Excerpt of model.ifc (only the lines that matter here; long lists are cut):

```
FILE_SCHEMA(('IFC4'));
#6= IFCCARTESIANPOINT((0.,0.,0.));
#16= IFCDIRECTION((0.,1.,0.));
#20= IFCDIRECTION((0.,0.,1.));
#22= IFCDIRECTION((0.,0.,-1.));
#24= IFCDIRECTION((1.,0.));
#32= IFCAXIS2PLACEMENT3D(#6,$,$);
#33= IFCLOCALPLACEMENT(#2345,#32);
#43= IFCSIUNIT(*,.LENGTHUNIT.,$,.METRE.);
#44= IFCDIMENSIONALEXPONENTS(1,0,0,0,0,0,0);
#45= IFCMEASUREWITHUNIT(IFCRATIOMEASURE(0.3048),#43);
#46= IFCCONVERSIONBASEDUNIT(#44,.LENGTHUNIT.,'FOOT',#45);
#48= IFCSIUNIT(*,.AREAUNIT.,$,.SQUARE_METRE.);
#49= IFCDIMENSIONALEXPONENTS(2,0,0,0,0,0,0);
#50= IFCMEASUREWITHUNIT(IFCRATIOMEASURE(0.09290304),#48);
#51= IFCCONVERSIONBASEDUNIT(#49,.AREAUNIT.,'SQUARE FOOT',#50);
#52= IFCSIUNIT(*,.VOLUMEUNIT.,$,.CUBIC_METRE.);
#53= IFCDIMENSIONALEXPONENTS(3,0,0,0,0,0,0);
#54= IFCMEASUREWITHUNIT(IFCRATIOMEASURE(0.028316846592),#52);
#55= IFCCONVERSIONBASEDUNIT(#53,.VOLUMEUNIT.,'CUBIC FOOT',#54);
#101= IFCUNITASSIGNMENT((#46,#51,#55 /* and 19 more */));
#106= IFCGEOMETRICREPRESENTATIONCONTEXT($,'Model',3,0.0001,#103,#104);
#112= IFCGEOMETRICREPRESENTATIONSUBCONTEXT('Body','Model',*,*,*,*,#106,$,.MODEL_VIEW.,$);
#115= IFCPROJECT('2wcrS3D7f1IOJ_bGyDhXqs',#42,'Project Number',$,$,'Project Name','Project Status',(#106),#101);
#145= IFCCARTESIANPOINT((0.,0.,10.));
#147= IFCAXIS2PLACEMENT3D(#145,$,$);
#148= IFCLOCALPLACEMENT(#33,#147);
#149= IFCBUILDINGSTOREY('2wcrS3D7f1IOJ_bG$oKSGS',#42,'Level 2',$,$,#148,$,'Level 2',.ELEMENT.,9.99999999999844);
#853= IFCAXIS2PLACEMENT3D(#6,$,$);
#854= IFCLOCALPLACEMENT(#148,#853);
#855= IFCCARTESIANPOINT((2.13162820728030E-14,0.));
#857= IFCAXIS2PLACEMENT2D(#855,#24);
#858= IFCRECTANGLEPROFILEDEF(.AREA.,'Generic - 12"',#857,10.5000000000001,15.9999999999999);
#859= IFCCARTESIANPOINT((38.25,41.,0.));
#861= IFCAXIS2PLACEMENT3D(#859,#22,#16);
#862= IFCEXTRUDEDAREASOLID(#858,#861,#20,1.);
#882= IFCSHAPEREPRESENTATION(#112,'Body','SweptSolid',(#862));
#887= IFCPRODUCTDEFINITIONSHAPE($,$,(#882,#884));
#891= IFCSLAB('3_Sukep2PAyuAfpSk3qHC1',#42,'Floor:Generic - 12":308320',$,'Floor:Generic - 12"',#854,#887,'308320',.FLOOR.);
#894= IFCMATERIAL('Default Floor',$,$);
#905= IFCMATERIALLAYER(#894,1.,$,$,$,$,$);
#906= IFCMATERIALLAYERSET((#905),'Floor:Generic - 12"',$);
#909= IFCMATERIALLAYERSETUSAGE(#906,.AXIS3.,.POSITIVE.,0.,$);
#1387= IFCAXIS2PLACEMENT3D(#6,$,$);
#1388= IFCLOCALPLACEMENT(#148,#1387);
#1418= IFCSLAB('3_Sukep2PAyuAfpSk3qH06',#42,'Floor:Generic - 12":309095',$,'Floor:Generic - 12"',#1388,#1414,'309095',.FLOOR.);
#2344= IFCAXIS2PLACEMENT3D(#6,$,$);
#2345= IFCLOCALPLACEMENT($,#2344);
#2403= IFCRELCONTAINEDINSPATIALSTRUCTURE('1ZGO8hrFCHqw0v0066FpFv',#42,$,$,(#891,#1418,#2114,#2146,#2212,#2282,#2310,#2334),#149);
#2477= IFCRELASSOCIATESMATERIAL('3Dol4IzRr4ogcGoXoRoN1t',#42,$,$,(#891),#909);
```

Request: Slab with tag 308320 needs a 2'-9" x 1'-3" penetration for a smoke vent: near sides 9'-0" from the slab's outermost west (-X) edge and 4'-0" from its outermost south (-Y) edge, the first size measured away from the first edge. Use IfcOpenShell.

```python
import numpy as np
import ifcopenshell
import ifcopenshell.api.feature
import ifcopenshell.api.geometry
import ifcopenshell.api.root
import ifcopenshell.geom
import ifcopenshell.util.placement
import ifcopenshell.util.representation
import ifcopenshell.util.shape
import ifcopenshell.util.unit

model = ifcopenshell.open("model.ifc")
unit_scale = ifcopenshell.util.unit.calculate_unit_scale(model)
settings = ifcopenshell.geom.settings()


def volume(element):
    """Net volume in cubic metres, openings subtracted."""
    shape = ifcopenshell.geom.create_shape(settings, element)
    return ifcopenshell.util.shape.get_volume(shape.geometry)


slab = model.by_guid("3_Sukep2PAyuAfpSk3qHC1")
before = volume(slab)

# Extent in the slab's own axes, in metres. The edges named are its -X and -Y sides.
slab_shape = ifcopenshell.geom.create_shape(settings, slab)
vertices = ifcopenshell.util.shape.get_vertices(slab_shape.geometry)
x_min, y_min, bottom = vertices.min(axis=0)
top = vertices[:, 2].max()

opening = ifcopenshell.api.root.create_entity(model, ifc_class="IfcOpeningElement", name="Smoke vent opening", predefined_type="OPENING")
context = ifcopenshell.util.representation.get_context(model, "Model", "Body", "MODEL_VIEW")
width, depth = 0.8382, 0.381
outline = [(0.0, 0.0), (width, 0.0), (width, depth), (0.0, depth), (0.0, 0.0)]
# Overshoot both faces by 50 mm so the cut is clean.
shape = ifcopenshell.api.geometry.add_slab_representation(
    model, context=context, depth=top - bottom + 0.1, polyline=outline
)
ifcopenshell.api.geometry.assign_representation(model, product=opening, representation=shape)

matrix = ifcopenshell.util.placement.get_local_placement(slab.ObjectPlacement)
matrix[:, 3] = matrix @ np.append(np.array([x_min + 2.7432, y_min + 1.2192, bottom - 0.05]) / unit_scale, 1.0)
ifcopenshell.api.geometry.edit_object_placement(model, product=opening, matrix=matrix, is_si=False)
ifcopenshell.api.feature.add_feature(model, feature=opening, element=slab)

after = volume(slab)

print(f"slab volume {before:.3f} -> {after:.3f} m3")

model.write("model_rev.ifc")
```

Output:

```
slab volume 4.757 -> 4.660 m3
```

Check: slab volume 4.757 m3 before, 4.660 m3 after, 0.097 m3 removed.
